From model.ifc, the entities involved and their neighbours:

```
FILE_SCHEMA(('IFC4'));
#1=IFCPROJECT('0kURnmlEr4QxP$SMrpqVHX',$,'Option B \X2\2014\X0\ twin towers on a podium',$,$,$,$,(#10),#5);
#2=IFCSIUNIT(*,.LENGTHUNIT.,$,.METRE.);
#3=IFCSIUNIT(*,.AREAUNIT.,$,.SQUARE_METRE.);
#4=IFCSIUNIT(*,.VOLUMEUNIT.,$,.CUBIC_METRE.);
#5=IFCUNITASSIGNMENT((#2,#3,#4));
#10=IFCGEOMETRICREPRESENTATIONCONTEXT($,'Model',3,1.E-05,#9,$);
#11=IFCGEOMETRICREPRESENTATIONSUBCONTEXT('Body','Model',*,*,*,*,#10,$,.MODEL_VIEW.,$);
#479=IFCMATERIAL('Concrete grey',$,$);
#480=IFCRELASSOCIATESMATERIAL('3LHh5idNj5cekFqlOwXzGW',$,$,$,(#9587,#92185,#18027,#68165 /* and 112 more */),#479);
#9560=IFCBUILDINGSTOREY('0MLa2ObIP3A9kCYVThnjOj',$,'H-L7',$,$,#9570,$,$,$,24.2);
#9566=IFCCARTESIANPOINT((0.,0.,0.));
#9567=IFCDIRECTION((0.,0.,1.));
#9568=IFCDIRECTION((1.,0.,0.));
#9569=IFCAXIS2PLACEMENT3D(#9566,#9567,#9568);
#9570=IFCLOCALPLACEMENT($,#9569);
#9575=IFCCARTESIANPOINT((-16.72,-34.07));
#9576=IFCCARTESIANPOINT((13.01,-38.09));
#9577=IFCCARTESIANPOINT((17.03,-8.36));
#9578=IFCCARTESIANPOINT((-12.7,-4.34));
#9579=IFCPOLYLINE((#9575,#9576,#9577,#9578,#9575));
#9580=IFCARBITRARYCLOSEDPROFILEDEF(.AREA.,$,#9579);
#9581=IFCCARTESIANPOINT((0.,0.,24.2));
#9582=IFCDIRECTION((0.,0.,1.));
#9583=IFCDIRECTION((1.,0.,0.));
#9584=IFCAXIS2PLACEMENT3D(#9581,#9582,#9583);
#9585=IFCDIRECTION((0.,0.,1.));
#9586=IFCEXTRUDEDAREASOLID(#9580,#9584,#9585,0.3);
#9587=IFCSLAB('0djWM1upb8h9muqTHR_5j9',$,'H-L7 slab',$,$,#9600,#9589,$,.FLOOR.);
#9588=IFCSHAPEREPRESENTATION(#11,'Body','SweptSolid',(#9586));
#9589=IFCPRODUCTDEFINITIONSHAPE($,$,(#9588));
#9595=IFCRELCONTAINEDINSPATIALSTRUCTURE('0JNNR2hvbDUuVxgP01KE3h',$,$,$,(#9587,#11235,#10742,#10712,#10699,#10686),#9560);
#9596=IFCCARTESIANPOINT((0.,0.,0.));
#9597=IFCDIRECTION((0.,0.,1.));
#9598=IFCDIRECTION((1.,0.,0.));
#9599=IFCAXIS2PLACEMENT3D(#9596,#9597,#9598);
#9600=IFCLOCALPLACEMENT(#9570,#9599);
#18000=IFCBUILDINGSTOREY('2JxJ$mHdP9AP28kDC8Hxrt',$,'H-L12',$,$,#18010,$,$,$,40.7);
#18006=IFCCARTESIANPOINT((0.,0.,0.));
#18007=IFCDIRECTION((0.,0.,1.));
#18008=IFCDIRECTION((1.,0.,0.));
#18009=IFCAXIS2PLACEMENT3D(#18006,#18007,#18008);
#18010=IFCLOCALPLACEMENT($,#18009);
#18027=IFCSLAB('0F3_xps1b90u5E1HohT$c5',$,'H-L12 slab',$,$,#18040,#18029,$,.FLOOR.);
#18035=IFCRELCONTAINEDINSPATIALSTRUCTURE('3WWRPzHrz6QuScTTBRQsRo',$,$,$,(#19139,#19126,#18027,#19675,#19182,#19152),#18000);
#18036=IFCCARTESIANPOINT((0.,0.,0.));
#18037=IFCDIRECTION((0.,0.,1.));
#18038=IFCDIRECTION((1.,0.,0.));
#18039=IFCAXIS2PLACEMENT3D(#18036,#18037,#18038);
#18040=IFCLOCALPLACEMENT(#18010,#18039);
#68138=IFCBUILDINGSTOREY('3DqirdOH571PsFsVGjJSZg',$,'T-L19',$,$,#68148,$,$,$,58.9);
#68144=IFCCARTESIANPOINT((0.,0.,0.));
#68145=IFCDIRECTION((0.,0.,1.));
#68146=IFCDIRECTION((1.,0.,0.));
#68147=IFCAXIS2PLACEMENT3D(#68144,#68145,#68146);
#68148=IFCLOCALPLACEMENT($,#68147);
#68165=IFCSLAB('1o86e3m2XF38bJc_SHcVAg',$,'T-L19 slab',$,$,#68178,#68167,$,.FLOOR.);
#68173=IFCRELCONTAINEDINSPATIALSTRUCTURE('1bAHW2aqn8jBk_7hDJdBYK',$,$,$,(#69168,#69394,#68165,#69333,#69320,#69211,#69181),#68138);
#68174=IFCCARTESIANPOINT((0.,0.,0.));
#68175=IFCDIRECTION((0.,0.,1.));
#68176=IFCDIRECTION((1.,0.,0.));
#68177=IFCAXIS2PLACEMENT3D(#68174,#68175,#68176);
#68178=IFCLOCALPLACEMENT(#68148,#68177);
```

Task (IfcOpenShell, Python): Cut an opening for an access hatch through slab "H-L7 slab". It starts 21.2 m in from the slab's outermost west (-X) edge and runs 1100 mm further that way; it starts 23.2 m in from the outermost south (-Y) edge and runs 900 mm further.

```python
import numpy as np
import ifcopenshell
import ifcopenshell.api.feature
import ifcopenshell.api.geometry
import ifcopenshell.api.root
import ifcopenshell.geom
import ifcopenshell.util.placement
import ifcopenshell.util.representation
import ifcopenshell.util.shape
import ifcopenshell.util.unit

model = ifcopenshell.open("model.ifc")
unit_scale = ifcopenshell.util.unit.calculate_unit_scale(model)
settings = ifcopenshell.geom.settings()


def volume(element):
    """Net volume in cubic metres, openings subtracted."""
    shape = ifcopenshell.geom.create_shape(settings, element)
    return ifcopenshell.util.shape.get_volume(shape.geometry)


slab = model.by_guid("0djWM1upb8h9muqTHR_5j9")
before = volume(slab)

# Extent in the slab's own axes, in metres. The edges named are its -X and -Y sides.
slab_shape = ifcopenshell.geom.create_shape(settings, slab)
vertices = ifcopenshell.util.shape.get_vertices(slab_shape.geometry)
x_min, y_min, bottom = vertices.min(axis=0)
top = vertices[:, 2].max()

opening = ifcopenshell.api.root.create_entity(model, ifc_class="IfcOpeningElement", name="Access hatch opening", predefined_type="OPENING")
context = ifcopenshell.util.representation.get_context(model, "Model", "Body", "MODEL_VIEW")
width, depth = 1.1, 0.9
outline = [(0.0, 0.0), (width, 0.0), (width, depth), (0.0, depth), (0.0, 0.0)]
# Overshoot both faces by 50 mm so the cut is clean.
shape = ifcopenshell.api.geometry.add_slab_representation(
    model, context=context, depth=top - bottom + 0.1, polyline=outline
)
ifcopenshell.api.geometry.assign_representation(model, product=opening, representation=shape)

matrix = ifcopenshell.util.placement.get_local_placement(slab.ObjectPlacement)
matrix[:, 3] = matrix @ np.append(np.array([x_min + 21.2, y_min + 23.2, bottom - 0.05]) / unit_scale, 1.0)
ifcopenshell.api.geometry.edit_object_placement(model, product=opening, matrix=matrix, is_si=False)
ifcopenshell.api.feature.add_feature(model, feature=opening, element=slab)

after = volume(slab)

print(f"slab volume {before:.3f} -> {after:.3f} m3")

model.write("model_updated.ifc")
```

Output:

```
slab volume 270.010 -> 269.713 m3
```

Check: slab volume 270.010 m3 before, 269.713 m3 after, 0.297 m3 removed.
